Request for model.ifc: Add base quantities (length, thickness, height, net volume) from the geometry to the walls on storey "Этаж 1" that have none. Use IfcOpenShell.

First a look at what the model holds.

```python
import ifcopenshell
import ifcopenshell.util.element
import ifcopenshell.util.unit

model = ifcopenshell.open("model.ifc")
print(model.schema)
for unit_type in ("LENGTHUNIT", "AREAUNIT", "VOLUMEUNIT"):
    print(unit_type, ifcopenshell.util.unit.calculate_unit_scale(model, unit_type))
storey = next(s for s in model.by_type("IfcBuildingStorey") if s.Name == "Этаж 1")
walls = [e for e in ifcopenshell.util.element.get_decomposition(storey) if e.is_a("IfcWall")]
for e in sorted(walls, key=lambda e: e.id()):
    print(e.id(), e.is_a(), e.Name, list(ifcopenshell.util.element.get_psets(e, qtos_only=True)), sep=" | ")
```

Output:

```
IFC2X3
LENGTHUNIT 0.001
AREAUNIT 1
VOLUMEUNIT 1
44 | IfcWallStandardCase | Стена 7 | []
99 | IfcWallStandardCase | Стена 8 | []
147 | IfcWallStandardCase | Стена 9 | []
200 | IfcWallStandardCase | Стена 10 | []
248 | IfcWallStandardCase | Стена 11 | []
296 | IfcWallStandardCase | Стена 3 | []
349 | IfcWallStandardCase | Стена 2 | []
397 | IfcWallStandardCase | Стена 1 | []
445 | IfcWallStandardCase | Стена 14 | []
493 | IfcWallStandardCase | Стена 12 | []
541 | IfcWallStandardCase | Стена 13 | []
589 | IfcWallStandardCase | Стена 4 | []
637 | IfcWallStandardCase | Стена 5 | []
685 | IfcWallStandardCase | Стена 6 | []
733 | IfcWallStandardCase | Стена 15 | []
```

```python
import ifcopenshell
import ifcopenshell.api.pset
import ifcopenshell.geom
import ifcopenshell.util.element
import ifcopenshell.util.shape
import ifcopenshell.util.unit

model = ifcopenshell.open("model.ifc")
unit_scale = ifcopenshell.util.unit.calculate_unit_scale(model)
volume_scale = ifcopenshell.util.unit.calculate_unit_scale(model, "VOLUMEUNIT")
settings = ifcopenshell.geom.settings()

storey = next(s for s in model.by_type("IfcBuildingStorey") if s.Name == "Этаж 1")
walls = [e for e in ifcopenshell.util.element.get_decomposition(storey) if e.is_a("IfcWall")]

for e in sorted(walls, key=lambda e: e.id()):
    if ifcopenshell.util.element.get_psets(e, qtos_only=True, should_inherit=False):
        continue
    # Geometry comes back in metres, in the element's own axes.
    shape = ifcopenshell.geom.create_shape(settings, e)
    values = {
        "Length": ifcopenshell.util.shape.get_x(shape.geometry) / unit_scale,
        "Width": ifcopenshell.util.shape.get_y(shape.geometry) / unit_scale,
        "Height": ifcopenshell.util.shape.get_z(shape.geometry) / unit_scale,
        "NetVolume": ifcopenshell.util.shape.get_volume(shape.geometry) / volume_scale,
    }
    qto = ifcopenshell.api.pset.add_qto(model, product=e, name="BaseQuantities")
    ifcopenshell.api.pset.edit_qto(model, qto=qto, properties=values)
    print(e.id(), {k: round(v, 3) for k, v in values.items()})

model.write("model-out.ifc")
```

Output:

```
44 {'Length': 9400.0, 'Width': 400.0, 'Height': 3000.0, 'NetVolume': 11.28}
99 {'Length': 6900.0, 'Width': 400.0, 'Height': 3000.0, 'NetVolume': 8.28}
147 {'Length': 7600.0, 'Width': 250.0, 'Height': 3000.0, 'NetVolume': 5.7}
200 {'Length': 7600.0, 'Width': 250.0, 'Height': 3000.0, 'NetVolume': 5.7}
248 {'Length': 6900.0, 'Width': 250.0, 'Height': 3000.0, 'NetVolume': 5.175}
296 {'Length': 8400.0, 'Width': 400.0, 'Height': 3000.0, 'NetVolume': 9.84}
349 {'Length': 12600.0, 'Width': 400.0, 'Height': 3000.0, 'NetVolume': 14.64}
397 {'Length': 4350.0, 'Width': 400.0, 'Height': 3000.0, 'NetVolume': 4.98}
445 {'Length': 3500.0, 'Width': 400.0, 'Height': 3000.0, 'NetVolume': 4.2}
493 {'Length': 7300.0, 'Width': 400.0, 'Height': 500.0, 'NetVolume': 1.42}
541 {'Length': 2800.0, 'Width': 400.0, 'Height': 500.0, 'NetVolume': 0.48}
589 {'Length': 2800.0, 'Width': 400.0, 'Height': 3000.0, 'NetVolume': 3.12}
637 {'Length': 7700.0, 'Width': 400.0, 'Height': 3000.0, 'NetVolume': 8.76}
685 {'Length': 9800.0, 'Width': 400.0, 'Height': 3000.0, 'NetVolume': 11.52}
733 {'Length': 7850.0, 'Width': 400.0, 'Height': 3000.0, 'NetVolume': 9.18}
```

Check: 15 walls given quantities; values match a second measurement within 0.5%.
